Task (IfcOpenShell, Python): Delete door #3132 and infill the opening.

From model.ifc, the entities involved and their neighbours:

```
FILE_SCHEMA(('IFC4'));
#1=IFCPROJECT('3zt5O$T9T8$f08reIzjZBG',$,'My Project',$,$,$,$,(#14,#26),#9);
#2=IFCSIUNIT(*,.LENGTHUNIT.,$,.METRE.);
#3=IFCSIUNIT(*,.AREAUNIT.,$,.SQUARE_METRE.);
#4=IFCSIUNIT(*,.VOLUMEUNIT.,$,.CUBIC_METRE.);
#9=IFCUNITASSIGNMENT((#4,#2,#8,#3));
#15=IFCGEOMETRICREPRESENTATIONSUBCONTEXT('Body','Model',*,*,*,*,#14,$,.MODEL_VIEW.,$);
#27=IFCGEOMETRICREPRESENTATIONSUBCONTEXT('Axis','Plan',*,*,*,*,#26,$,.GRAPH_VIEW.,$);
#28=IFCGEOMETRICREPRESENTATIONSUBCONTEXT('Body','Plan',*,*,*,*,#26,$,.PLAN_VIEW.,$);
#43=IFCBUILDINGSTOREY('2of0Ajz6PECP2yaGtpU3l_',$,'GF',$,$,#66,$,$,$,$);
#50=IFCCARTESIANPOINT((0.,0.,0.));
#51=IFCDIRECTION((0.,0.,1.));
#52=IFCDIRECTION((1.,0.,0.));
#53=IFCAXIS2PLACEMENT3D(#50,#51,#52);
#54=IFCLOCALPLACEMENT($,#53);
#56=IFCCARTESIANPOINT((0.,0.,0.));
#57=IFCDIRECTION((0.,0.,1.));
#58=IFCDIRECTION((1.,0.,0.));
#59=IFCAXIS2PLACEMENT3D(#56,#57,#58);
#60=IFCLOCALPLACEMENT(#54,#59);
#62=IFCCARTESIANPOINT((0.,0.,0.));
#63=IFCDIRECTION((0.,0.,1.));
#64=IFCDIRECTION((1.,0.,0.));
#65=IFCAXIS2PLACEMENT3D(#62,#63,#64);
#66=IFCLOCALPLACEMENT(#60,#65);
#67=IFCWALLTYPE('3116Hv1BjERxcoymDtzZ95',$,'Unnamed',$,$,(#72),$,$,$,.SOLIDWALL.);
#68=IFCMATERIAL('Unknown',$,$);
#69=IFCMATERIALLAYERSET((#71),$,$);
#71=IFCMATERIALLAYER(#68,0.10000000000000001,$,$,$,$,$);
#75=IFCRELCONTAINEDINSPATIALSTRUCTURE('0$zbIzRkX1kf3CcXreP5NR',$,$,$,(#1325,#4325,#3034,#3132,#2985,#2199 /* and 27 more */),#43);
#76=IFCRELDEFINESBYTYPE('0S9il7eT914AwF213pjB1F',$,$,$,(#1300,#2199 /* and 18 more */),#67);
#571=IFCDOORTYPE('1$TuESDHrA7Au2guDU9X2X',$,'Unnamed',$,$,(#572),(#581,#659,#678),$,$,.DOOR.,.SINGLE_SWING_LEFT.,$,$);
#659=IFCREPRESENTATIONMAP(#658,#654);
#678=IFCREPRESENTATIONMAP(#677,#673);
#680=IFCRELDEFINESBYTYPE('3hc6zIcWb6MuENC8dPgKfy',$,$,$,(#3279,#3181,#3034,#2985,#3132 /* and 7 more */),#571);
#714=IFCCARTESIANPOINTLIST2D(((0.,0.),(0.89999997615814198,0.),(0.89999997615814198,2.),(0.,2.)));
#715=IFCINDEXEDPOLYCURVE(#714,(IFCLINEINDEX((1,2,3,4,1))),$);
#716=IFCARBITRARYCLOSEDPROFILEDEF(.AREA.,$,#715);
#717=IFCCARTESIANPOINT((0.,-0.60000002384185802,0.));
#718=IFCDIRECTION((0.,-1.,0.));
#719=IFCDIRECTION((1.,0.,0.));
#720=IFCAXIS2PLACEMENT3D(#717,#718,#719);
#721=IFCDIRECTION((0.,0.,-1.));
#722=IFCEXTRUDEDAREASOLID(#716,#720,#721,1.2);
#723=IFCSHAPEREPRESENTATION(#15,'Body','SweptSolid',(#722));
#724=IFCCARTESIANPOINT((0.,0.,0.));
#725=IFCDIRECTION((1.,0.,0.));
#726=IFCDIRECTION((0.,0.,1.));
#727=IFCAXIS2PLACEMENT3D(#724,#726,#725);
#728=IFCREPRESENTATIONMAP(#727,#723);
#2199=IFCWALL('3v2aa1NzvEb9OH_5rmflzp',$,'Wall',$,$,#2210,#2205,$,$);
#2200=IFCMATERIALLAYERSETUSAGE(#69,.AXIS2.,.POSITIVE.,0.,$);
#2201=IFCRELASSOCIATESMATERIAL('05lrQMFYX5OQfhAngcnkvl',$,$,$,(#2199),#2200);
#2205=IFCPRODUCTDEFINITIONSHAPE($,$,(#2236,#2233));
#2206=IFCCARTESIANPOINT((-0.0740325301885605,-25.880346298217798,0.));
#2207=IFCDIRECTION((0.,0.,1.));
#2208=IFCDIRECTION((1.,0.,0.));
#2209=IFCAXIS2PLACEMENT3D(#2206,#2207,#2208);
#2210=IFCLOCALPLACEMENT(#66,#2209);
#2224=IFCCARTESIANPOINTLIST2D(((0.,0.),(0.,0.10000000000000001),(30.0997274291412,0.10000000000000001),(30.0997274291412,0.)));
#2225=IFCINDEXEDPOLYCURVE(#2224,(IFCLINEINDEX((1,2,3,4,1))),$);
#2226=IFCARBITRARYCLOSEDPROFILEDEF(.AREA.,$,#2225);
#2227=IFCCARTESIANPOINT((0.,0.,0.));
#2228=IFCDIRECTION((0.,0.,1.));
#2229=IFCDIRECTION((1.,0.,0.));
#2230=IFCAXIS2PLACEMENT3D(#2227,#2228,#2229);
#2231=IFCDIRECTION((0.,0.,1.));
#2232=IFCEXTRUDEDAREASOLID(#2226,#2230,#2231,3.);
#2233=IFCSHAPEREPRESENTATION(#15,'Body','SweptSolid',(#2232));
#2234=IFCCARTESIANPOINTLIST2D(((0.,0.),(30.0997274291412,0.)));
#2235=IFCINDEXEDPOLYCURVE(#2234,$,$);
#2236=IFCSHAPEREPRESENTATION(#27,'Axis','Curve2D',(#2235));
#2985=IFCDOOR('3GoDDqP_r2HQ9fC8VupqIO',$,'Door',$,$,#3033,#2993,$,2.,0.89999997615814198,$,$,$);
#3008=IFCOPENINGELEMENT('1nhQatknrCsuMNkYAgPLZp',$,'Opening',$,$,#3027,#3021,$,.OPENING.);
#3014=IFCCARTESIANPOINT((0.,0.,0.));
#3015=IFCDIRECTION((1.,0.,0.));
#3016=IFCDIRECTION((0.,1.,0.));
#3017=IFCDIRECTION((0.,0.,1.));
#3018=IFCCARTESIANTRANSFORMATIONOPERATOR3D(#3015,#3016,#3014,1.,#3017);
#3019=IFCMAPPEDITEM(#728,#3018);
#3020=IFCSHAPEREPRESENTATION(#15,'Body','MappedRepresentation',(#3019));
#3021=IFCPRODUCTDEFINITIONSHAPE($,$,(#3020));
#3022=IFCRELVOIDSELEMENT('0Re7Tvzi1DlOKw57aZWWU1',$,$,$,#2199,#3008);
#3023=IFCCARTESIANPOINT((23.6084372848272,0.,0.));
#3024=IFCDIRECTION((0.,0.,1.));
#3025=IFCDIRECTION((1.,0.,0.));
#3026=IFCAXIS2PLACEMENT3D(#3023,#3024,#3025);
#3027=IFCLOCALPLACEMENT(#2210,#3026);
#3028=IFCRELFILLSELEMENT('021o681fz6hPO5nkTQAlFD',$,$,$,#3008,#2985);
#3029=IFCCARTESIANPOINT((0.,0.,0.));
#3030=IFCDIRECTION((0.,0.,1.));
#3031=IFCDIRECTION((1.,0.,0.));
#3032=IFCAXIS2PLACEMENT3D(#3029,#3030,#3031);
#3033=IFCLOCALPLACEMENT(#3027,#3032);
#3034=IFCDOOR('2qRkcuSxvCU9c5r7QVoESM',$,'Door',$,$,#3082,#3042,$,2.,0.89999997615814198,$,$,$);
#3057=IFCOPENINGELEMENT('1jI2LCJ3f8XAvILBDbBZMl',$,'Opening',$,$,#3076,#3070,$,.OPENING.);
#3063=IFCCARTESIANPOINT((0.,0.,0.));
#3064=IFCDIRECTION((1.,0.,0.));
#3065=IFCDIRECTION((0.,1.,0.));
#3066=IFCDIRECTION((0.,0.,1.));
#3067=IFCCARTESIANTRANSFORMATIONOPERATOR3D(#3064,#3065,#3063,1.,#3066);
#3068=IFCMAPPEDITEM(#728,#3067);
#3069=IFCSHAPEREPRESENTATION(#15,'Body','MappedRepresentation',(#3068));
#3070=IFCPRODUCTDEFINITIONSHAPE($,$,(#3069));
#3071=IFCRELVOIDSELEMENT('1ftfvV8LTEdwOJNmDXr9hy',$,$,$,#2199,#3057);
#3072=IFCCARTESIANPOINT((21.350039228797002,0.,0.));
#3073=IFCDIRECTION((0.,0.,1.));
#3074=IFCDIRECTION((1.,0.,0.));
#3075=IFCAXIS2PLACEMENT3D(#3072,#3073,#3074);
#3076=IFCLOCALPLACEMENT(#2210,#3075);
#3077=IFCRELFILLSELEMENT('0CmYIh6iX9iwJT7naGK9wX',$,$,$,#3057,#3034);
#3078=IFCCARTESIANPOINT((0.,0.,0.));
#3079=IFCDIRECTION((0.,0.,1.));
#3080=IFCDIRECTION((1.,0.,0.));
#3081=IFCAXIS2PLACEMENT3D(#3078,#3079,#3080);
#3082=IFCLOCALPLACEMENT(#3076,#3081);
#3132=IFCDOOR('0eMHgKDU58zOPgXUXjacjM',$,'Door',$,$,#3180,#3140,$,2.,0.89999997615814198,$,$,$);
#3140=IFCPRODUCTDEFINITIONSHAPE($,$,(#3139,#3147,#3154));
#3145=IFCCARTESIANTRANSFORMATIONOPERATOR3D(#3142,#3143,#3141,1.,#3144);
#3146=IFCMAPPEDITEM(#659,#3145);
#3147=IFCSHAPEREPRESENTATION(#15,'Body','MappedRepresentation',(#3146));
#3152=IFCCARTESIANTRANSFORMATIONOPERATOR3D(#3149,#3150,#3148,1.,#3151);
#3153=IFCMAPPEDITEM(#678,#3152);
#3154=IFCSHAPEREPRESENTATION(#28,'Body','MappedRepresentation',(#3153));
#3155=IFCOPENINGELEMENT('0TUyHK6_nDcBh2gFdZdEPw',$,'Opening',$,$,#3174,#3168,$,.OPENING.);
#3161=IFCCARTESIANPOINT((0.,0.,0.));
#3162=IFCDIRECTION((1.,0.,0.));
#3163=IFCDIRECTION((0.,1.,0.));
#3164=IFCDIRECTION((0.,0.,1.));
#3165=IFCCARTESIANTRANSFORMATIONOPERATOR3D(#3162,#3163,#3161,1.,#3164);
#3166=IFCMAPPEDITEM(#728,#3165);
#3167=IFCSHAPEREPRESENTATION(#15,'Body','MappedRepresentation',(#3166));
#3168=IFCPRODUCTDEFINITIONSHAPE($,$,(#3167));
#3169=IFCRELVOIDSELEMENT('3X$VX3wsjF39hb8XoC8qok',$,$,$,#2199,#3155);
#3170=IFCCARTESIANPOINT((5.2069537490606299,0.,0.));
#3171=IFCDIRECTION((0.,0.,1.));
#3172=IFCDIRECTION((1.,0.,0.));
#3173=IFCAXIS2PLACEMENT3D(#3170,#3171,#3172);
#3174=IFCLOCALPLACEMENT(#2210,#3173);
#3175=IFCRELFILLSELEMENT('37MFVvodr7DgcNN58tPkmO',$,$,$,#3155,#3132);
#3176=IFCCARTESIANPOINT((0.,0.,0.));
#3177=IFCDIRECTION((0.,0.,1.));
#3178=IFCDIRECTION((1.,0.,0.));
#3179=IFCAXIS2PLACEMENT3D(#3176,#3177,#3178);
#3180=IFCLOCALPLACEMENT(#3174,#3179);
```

```python
import ifcopenshell
import ifcopenshell.api.feature
import ifcopenshell.api.root
import ifcopenshell.geom
import ifcopenshell.util.shape

model = ifcopenshell.open("model.ifc")
settings = ifcopenshell.geom.settings()


def volume(element):
    """Net volume in cubic metres, openings subtracted."""
    shape = ifcopenshell.geom.create_shape(settings, element)
    return ifcopenshell.util.shape.get_volume(shape.geometry)


door = model.by_id(3132)
opening = door.FillsVoids[0].RelatingOpeningElement
wall = opening.VoidsElements[0].RelatingBuildingElement
before = volume(wall)

ifcopenshell.api.root.remove_product(model, product=door)
ifcopenshell.api.feature.remove_feature(model, feature=opening)

after = volume(wall)

print(f"wall volume {before:.3f} -> {after:.3f} m3")

model.write("model-out.ifc")
```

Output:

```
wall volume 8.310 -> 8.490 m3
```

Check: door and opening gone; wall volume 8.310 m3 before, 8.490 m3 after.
